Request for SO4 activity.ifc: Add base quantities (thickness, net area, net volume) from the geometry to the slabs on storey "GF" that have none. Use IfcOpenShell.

First a look at what the model holds.

```python
import ifcopenshell
import ifcopenshell.util.element
import ifcopenshell.util.unit

model = ifcopenshell.open("SO4 activity.ifc")
print(model.schema)
for unit_type in ("LENGTHUNIT", "AREAUNIT", "VOLUMEUNIT"):
    print(unit_type, ifcopenshell.util.unit.calculate_unit_scale(model, unit_type))
storey = next(s for s in model.by_type("IfcBuildingStorey") if s.Name == "GF")
slabs = [e for e in ifcopenshell.util.element.get_decomposition(storey) if e.is_a("IfcSlab")]
for e in sorted(slabs, key=lambda e: e.id()):
    print(e.id(), e.is_a(), e.Name, list(ifcopenshell.util.element.get_psets(e, qtos_only=True)), sep=" | ")
```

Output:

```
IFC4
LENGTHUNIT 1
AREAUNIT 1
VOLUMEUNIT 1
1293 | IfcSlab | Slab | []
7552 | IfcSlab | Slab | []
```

```python
import ifcopenshell
import ifcopenshell.api.pset
import ifcopenshell.geom
import ifcopenshell.util.element
import ifcopenshell.util.shape
import ifcopenshell.util.unit

model = ifcopenshell.open("SO4 activity.ifc")
unit_scale = ifcopenshell.util.unit.calculate_unit_scale(model)
area_scale = ifcopenshell.util.unit.calculate_unit_scale(model, "AREAUNIT")
volume_scale = ifcopenshell.util.unit.calculate_unit_scale(model, "VOLUMEUNIT")
settings = ifcopenshell.geom.settings()

storey = next(s for s in model.by_type("IfcBuildingStorey") if s.Name == "GF")
slabs = [e for e in ifcopenshell.util.element.get_decomposition(storey) if e.is_a("IfcSlab")]

for e in sorted(slabs, key=lambda e: e.id()):
    if ifcopenshell.util.element.get_psets(e, qtos_only=True, should_inherit=False):
        continue
    # Geometry comes back in metres, in the element's own axes.
    shape = ifcopenshell.geom.create_shape(settings, e)
    values = {
        "Width": ifcopenshell.util.shape.get_z(shape.geometry) / unit_scale,
        "NetArea": ifcopenshell.util.shape.get_footprint_area(shape.geometry) / area_scale,
        "NetVolume": ifcopenshell.util.shape.get_volume(shape.geometry) / volume_scale,
    }
    qto = ifcopenshell.api.pset.add_qto(model, product=e, name="Qto_SlabBaseQuantities")
    ifcopenshell.api.pset.edit_qto(model, qto=qto, properties=values)
    print(e.id(), {k: round(v, 3) for k, v in values.items()})

model.write("SO4 activity_rev.ifc")
```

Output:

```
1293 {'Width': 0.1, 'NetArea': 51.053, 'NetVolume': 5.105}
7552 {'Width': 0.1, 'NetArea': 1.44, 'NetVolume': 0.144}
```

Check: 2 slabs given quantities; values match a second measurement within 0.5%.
